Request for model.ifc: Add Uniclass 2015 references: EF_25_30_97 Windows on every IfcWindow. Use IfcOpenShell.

First a look at what the model holds.

```python
import ifcopenshell

model = ifcopenshell.open("model.ifc")
print(model.schema)
print("classifications:", [c.Name for c in model.by_type("IfcClassification")])
for ifc_class in ("IfcDoor", "IfcRoof", "IfcStair", "IfcWall", "IfcWindow"):
    print(ifc_class, len(model.by_type(ifc_class)))
```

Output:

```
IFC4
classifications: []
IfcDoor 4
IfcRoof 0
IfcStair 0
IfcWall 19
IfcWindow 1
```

```python
import ifcopenshell
import ifcopenshell.api.classification

model = ifcopenshell.open("model.ifc")

system = ifcopenshell.api.classification.add_classification(model, classification="Uniclass 2015")

codes = {
    "IfcWindow": ("EF_25_30_97", "Windows"),
}
for ifc_class, (code, name) in codes.items():
    products = model.by_type(ifc_class)
    ifcopenshell.api.classification.add_reference(
        model, products=products, classification=system, identification=code, name=name
    )
    print(code, len(products))

model.write("model_rev.ifc")
```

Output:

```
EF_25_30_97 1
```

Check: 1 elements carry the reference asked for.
